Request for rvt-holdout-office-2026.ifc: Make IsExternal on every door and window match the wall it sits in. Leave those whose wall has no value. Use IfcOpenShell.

First a look at what the model holds.

```python
import ifcopenshell
import ifcopenshell.util.element

model = ifcopenshell.open("rvt-holdout-office-2026.ifc")
print(model.schema)
seen = {}
for e in model.by_type("IfcDoor") + model.by_type("IfcWindow"):
    if not e.FillsVoids:
        continue
    host = e.FillsVoids[0].RelatingOpeningElement.VoidsElements[0].RelatingBuildingElement
    own = ifcopenshell.util.element.get_pset(e, f"Pset_{e.is_a()[3:].removesuffix('StandardCase')}Common", "IsExternal")
    wall = ifcopenshell.util.element.get_pset(host, "Pset_WallCommon", "IsExternal")
    seen[e.is_a(), own, wall] = seen.get((e.is_a(), own, wall), 0) + 1
for (cls, own, wall), count in sorted(seen.items(), key=str):
    print(count, cls, "IsExternal:", own, "| host wall:", wall)
```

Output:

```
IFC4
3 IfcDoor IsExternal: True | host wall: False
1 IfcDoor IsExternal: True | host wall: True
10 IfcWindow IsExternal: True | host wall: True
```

```python
import ifcopenshell
import ifcopenshell.api.pset
import ifcopenshell.util.element

model = ifcopenshell.open("rvt-holdout-office-2026.ifc")

count = 0
for ifc_class, pset_name in (("IfcDoor", "Pset_DoorCommon"), ("IfcWindow", "Pset_WindowCommon")):
    for e in model.by_type(ifc_class):
        if not e.FillsVoids:
            continue
        host = e.FillsVoids[0].RelatingOpeningElement.VoidsElements[0].RelatingBuildingElement
        external = ifcopenshell.util.element.get_pset(host, "Pset_WallCommon", "IsExternal")
        if external is None or ifcopenshell.util.element.get_pset(e, pset_name, "IsExternal") == external:
            continue
        pset = ifcopenshell.api.pset.add_pset(model, product=e, name=pset_name)
        ifcopenshell.api.pset.edit_pset(model, pset=pset, properties={"IsExternal": external})
        count += 1

print(count, "updated")

model.write("rvt-holdout-office-2026_v2.ifc")
```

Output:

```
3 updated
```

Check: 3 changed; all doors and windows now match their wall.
